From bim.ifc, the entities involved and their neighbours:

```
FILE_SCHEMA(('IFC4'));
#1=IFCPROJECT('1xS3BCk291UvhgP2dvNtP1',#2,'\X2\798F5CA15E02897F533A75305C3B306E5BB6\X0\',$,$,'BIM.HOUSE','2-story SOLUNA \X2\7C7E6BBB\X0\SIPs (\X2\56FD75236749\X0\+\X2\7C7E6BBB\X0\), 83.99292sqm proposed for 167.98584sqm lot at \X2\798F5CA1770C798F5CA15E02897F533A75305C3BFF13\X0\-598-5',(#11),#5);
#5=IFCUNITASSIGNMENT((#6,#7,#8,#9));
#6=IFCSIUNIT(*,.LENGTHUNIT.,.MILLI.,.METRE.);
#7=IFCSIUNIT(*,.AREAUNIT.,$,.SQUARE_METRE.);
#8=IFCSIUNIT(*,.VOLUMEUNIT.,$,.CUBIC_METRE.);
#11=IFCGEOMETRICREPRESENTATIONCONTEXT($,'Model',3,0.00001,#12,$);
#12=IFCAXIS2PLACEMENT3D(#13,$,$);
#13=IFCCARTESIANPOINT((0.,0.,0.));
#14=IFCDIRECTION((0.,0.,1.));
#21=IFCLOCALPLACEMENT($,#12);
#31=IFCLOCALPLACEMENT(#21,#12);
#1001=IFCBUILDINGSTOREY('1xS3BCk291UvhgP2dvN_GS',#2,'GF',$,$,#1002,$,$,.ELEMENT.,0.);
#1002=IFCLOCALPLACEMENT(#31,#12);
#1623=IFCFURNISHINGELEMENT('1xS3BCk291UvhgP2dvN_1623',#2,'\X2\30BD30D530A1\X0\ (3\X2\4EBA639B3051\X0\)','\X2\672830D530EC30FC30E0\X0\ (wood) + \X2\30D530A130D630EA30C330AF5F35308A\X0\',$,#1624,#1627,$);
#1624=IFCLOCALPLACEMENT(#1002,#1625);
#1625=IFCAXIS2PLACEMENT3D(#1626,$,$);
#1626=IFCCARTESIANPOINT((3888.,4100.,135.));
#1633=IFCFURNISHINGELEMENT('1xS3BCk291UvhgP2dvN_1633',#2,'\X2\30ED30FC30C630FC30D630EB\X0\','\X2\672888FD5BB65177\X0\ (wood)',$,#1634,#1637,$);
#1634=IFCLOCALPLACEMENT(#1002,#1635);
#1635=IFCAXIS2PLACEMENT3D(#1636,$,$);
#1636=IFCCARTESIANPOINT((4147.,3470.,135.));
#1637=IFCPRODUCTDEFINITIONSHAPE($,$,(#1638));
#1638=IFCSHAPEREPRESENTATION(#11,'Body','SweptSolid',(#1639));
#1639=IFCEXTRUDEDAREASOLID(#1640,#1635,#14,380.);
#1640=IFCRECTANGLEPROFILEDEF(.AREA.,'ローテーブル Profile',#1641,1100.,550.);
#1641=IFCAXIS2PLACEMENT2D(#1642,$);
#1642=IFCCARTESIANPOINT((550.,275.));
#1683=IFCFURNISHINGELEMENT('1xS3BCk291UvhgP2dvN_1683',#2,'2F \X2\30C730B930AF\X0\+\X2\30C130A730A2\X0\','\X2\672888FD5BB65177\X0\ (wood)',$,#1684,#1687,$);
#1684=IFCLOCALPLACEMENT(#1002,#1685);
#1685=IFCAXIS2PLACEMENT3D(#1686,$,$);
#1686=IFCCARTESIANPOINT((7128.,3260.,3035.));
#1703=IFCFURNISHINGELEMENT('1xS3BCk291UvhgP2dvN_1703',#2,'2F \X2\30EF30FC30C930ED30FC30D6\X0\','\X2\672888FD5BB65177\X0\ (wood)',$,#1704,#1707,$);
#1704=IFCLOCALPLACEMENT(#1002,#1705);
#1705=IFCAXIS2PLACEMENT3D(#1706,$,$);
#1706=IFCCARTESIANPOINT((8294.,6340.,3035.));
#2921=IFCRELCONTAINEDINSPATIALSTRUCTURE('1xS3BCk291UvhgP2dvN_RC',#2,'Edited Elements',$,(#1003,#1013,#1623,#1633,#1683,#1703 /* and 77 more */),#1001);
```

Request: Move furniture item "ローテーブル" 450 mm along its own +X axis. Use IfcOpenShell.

```python
import ifcopenshell
import ifcopenshell.api.geometry
import ifcopenshell.util.placement

model = ifcopenshell.open("bim.ifc")

item = model.by_id(1633)
matrix = ifcopenshell.util.placement.get_local_placement(item.ObjectPlacement)
matrix[:3, 3] += matrix[:3, 0] * 450.0
ifcopenshell.api.geometry.edit_object_placement(model, product=item, matrix=matrix, is_si=False)

print(ifcopenshell.util.placement.get_local_placement(item.ObjectPlacement).round(3) + 0.0)

model.write("bim_v2.ifc")
```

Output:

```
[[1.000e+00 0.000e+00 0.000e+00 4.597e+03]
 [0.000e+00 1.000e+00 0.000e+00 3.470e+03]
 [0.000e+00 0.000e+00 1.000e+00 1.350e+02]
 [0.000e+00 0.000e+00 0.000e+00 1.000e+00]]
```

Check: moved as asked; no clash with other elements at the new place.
